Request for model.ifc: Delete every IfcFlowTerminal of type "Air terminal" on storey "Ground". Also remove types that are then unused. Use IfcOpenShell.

First a look at what the model holds.

```python
import ifcopenshell
import ifcopenshell.util.element

model = ifcopenshell.open("model.ifc")
print(model.schema)
storey = next(s for s in model.by_type("IfcBuildingStorey") if s.Name == "Ground")
terminals = [e for e in ifcopenshell.util.element.get_decomposition(storey) if e.is_a("IfcFlowTerminal")]
seen = {}
for e in terminals:
    element_type = ifcopenshell.util.element.get_type(e)
    name = element_type.Name if element_type not in (None, e) else None
    seen[name] = seen.get(name, 0) + 1
for name, count in sorted(seen.items(), key=str):
    print(count, "x", name)
```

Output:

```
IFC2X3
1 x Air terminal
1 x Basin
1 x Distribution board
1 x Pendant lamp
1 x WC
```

```python
import ifcopenshell
import ifcopenshell.api.root
import ifcopenshell.util.element

model = ifcopenshell.open("model.ifc")

storey = next(s for s in model.by_type("IfcBuildingStorey") if s.Name == "Ground")
terminals = [e for e in ifcopenshell.util.element.get_decomposition(storey) if e.is_a("IfcFlowTerminal")]
targets = [e for e in terminals if (t := ifcopenshell.util.element.get_type(e)) not in (None, e) and t.Name == "Air terminal"]
types = {ifcopenshell.util.element.get_type(e) for e in targets} - {None, *targets}

for e in targets:
    ifcopenshell.api.root.remove_product(model, product=e)
print(len(targets), "removed")

unused = [t for t in types if not ifcopenshell.util.element.get_types(t)]
for t in unused:
    ifcopenshell.api.root.remove_product(model, product=t)
print(len(unused), "unused types removed")

model.write("model_rev.ifc")
```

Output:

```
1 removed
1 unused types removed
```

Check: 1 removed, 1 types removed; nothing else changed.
